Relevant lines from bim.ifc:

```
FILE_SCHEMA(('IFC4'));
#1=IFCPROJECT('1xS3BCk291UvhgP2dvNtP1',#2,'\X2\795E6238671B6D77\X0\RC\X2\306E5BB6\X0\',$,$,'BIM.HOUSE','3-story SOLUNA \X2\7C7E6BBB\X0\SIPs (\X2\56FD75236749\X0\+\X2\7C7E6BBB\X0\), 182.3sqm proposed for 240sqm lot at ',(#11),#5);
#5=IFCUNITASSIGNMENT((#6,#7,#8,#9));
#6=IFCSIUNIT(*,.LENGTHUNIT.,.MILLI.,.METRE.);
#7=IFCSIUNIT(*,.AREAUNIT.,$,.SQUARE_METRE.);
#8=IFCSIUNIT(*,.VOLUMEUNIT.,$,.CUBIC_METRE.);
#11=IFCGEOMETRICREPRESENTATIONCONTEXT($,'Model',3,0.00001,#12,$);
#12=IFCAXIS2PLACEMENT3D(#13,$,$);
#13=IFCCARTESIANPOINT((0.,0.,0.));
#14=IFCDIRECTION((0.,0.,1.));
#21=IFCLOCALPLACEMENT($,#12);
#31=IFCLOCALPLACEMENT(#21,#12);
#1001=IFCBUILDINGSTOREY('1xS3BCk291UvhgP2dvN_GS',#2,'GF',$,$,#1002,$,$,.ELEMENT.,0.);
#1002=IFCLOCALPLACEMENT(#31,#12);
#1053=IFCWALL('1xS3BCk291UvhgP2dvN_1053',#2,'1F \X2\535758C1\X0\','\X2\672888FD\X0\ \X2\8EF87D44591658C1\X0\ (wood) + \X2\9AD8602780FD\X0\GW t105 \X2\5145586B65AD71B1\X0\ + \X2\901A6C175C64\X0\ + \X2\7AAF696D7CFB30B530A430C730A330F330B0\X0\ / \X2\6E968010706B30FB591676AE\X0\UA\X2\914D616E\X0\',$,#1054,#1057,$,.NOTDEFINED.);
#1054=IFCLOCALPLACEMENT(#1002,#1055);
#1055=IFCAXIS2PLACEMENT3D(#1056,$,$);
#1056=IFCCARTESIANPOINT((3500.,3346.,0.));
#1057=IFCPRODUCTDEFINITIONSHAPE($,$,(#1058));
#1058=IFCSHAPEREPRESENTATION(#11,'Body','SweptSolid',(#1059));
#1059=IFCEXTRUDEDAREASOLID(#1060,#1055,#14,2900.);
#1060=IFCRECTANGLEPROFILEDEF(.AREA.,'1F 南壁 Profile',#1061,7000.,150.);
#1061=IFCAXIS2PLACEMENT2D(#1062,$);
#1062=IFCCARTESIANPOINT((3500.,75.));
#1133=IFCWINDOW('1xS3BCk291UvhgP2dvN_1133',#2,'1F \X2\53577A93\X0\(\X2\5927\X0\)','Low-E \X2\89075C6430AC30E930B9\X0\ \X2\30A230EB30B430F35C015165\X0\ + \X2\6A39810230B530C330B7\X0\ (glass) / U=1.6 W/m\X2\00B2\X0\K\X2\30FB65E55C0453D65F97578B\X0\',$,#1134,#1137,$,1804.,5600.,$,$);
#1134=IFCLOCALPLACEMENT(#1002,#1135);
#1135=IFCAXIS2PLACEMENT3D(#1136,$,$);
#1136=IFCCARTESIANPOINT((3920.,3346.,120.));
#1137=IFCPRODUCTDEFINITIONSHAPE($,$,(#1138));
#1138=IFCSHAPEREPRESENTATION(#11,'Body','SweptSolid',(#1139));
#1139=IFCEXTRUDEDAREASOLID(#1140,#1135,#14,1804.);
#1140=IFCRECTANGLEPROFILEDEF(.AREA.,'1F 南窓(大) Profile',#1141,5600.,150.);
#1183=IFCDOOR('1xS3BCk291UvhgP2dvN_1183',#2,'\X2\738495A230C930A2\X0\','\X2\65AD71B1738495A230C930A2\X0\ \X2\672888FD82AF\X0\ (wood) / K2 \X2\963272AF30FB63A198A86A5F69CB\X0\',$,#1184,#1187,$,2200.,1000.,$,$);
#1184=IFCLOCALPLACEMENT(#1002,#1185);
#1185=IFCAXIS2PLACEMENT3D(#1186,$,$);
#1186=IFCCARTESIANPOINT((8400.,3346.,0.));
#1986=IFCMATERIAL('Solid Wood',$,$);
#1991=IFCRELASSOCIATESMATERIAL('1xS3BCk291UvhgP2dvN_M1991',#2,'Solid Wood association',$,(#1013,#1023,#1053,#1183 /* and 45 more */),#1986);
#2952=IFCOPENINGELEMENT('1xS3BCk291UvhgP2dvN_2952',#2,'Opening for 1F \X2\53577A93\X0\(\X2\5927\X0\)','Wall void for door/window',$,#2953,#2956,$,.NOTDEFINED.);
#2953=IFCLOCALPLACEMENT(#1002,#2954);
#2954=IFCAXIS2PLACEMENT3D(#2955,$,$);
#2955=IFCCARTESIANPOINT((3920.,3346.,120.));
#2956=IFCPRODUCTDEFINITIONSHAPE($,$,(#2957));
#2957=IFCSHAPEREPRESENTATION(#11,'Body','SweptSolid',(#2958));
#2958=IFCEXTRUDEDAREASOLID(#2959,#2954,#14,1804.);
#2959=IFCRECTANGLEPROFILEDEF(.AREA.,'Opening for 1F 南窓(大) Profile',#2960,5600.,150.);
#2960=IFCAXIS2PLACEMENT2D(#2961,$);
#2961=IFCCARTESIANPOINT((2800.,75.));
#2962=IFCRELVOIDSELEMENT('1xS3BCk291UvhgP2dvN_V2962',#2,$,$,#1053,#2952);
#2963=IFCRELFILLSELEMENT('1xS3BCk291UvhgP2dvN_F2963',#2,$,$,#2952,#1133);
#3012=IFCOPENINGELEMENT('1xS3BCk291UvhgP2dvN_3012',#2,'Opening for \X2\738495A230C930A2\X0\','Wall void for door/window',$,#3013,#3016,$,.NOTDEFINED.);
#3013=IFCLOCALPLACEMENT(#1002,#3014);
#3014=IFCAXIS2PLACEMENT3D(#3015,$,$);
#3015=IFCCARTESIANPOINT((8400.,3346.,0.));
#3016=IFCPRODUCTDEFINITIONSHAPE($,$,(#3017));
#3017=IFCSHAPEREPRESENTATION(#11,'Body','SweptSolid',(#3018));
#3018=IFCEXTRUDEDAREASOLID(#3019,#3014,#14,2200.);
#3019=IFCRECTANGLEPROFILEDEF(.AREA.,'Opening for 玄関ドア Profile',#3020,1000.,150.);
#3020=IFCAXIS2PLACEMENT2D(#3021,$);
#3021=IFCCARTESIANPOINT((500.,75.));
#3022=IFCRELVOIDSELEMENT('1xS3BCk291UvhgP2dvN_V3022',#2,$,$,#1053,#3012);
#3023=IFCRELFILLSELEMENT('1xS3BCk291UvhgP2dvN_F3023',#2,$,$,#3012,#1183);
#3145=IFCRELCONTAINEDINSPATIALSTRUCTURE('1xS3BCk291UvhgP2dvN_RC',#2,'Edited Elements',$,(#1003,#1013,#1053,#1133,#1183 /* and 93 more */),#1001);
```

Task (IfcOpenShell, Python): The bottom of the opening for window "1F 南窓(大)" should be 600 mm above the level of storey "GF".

```python
import numpy as np
import ifcopenshell
import ifcopenshell.api.geometry
import ifcopenshell.geom
import ifcopenshell.util.element
import ifcopenshell.util.placement
import ifcopenshell.util.shape
import ifcopenshell.util.unit

model = ifcopenshell.open("bim.ifc")
unit_scale = ifcopenshell.util.unit.calculate_unit_scale(model)

window = model.by_guid("1xS3BCk291UvhgP2dvN_1133")
opening = window.FillsVoids[0].RelatingOpeningElement
storey = ifcopenshell.util.element.get_container(window, ifc_class="IfcBuildingStorey")
level = ifcopenshell.util.placement.get_local_placement(storey.ObjectPlacement)[2, 3]

# The opening's origin need not be at the sill, so measure its lowest point.
shape = ifcopenshell.geom.create_shape(ifcopenshell.geom.settings(), opening)
bottom = ifcopenshell.util.shape.get_shape_bottom_elevation(shape, shape.geometry) / unit_scale
dz = level + 0.6 / unit_scale - bottom

shift = np.array([0.0, 0.0, dz])
# The window is not placed relative to its opening, so move both.
for product in (opening, window):
    matrix = ifcopenshell.util.placement.get_local_placement(product.ObjectPlacement)
    matrix[:3, 3] += shift
    ifcopenshell.api.geometry.edit_object_placement(model, product=product, matrix=matrix, is_si=False)

print(f"moved by {dz * unit_scale:+.3f} m")

model.write("bim_edited.ifc")
```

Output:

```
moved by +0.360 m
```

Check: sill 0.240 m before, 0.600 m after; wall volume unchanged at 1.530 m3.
